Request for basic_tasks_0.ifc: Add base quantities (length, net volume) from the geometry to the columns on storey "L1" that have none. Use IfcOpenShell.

First a look at what the model holds.

```python
import ifcopenshell
import ifcopenshell.util.element
import ifcopenshell.util.unit

model = ifcopenshell.open("basic_tasks_0.ifc")
print(model.schema)
for unit_type in ("LENGTHUNIT", "AREAUNIT", "VOLUMEUNIT"):
    print(unit_type, ifcopenshell.util.unit.calculate_unit_scale(model, unit_type))
storey = next(s for s in model.by_type("IfcBuildingStorey") if s.Name == "L1")
columns = [e for e in ifcopenshell.util.element.get_decomposition(storey) if e.is_a("IfcColumn")]
for e in sorted(columns, key=lambda e: e.id()):
    print(e.id(), e.is_a(), e.Name, list(ifcopenshell.util.element.get_psets(e, qtos_only=True)), sep=" | ")
```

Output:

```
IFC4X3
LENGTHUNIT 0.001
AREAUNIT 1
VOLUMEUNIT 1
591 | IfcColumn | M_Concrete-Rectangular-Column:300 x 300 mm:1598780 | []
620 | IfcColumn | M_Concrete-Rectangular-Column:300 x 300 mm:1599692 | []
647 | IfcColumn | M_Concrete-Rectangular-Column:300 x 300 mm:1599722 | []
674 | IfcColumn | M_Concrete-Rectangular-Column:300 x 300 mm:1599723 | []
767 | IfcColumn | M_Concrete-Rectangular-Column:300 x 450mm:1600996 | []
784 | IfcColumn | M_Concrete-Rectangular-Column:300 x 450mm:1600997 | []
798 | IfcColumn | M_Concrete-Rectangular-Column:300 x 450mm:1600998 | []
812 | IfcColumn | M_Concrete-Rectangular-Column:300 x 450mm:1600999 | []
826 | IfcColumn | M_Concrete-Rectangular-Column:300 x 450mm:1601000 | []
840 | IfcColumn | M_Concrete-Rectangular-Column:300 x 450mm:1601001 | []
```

```python
import ifcopenshell
import ifcopenshell.api.pset
import ifcopenshell.geom
import ifcopenshell.util.element
import ifcopenshell.util.shape
import ifcopenshell.util.unit

model = ifcopenshell.open("basic_tasks_0.ifc")
unit_scale = ifcopenshell.util.unit.calculate_unit_scale(model)
volume_scale = ifcopenshell.util.unit.calculate_unit_scale(model, "VOLUMEUNIT")
settings = ifcopenshell.geom.settings()

storey = next(s for s in model.by_type("IfcBuildingStorey") if s.Name == "L1")
columns = [e for e in ifcopenshell.util.element.get_decomposition(storey) if e.is_a("IfcColumn")]

for e in sorted(columns, key=lambda e: e.id()):
    if ifcopenshell.util.element.get_psets(e, qtos_only=True, should_inherit=False):
        continue
    # Geometry comes back in metres, in the element's own axes.
    shape = ifcopenshell.geom.create_shape(settings, e)
    values = {
        "Length": ifcopenshell.util.shape.get_z(shape.geometry) / unit_scale,
        "NetVolume": ifcopenshell.util.shape.get_volume(shape.geometry) / volume_scale,
    }
    qto = ifcopenshell.api.pset.add_qto(model, product=e, name="Qto_ColumnBaseQuantities")
    ifcopenshell.api.pset.edit_qto(model, qto=qto, properties=values)
    print(e.id(), {k: round(v, 3) for k, v in values.items()})

model.write("basic_tasks_0_rev.ifc")
```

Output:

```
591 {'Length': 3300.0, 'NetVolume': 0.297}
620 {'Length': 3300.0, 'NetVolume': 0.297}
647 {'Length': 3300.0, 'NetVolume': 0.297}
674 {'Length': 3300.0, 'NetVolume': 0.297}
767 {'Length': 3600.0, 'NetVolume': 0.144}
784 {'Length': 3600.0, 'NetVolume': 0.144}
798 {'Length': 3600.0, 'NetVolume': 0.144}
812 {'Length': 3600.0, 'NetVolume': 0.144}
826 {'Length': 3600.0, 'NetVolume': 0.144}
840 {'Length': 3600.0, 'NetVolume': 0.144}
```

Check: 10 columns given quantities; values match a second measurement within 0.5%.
